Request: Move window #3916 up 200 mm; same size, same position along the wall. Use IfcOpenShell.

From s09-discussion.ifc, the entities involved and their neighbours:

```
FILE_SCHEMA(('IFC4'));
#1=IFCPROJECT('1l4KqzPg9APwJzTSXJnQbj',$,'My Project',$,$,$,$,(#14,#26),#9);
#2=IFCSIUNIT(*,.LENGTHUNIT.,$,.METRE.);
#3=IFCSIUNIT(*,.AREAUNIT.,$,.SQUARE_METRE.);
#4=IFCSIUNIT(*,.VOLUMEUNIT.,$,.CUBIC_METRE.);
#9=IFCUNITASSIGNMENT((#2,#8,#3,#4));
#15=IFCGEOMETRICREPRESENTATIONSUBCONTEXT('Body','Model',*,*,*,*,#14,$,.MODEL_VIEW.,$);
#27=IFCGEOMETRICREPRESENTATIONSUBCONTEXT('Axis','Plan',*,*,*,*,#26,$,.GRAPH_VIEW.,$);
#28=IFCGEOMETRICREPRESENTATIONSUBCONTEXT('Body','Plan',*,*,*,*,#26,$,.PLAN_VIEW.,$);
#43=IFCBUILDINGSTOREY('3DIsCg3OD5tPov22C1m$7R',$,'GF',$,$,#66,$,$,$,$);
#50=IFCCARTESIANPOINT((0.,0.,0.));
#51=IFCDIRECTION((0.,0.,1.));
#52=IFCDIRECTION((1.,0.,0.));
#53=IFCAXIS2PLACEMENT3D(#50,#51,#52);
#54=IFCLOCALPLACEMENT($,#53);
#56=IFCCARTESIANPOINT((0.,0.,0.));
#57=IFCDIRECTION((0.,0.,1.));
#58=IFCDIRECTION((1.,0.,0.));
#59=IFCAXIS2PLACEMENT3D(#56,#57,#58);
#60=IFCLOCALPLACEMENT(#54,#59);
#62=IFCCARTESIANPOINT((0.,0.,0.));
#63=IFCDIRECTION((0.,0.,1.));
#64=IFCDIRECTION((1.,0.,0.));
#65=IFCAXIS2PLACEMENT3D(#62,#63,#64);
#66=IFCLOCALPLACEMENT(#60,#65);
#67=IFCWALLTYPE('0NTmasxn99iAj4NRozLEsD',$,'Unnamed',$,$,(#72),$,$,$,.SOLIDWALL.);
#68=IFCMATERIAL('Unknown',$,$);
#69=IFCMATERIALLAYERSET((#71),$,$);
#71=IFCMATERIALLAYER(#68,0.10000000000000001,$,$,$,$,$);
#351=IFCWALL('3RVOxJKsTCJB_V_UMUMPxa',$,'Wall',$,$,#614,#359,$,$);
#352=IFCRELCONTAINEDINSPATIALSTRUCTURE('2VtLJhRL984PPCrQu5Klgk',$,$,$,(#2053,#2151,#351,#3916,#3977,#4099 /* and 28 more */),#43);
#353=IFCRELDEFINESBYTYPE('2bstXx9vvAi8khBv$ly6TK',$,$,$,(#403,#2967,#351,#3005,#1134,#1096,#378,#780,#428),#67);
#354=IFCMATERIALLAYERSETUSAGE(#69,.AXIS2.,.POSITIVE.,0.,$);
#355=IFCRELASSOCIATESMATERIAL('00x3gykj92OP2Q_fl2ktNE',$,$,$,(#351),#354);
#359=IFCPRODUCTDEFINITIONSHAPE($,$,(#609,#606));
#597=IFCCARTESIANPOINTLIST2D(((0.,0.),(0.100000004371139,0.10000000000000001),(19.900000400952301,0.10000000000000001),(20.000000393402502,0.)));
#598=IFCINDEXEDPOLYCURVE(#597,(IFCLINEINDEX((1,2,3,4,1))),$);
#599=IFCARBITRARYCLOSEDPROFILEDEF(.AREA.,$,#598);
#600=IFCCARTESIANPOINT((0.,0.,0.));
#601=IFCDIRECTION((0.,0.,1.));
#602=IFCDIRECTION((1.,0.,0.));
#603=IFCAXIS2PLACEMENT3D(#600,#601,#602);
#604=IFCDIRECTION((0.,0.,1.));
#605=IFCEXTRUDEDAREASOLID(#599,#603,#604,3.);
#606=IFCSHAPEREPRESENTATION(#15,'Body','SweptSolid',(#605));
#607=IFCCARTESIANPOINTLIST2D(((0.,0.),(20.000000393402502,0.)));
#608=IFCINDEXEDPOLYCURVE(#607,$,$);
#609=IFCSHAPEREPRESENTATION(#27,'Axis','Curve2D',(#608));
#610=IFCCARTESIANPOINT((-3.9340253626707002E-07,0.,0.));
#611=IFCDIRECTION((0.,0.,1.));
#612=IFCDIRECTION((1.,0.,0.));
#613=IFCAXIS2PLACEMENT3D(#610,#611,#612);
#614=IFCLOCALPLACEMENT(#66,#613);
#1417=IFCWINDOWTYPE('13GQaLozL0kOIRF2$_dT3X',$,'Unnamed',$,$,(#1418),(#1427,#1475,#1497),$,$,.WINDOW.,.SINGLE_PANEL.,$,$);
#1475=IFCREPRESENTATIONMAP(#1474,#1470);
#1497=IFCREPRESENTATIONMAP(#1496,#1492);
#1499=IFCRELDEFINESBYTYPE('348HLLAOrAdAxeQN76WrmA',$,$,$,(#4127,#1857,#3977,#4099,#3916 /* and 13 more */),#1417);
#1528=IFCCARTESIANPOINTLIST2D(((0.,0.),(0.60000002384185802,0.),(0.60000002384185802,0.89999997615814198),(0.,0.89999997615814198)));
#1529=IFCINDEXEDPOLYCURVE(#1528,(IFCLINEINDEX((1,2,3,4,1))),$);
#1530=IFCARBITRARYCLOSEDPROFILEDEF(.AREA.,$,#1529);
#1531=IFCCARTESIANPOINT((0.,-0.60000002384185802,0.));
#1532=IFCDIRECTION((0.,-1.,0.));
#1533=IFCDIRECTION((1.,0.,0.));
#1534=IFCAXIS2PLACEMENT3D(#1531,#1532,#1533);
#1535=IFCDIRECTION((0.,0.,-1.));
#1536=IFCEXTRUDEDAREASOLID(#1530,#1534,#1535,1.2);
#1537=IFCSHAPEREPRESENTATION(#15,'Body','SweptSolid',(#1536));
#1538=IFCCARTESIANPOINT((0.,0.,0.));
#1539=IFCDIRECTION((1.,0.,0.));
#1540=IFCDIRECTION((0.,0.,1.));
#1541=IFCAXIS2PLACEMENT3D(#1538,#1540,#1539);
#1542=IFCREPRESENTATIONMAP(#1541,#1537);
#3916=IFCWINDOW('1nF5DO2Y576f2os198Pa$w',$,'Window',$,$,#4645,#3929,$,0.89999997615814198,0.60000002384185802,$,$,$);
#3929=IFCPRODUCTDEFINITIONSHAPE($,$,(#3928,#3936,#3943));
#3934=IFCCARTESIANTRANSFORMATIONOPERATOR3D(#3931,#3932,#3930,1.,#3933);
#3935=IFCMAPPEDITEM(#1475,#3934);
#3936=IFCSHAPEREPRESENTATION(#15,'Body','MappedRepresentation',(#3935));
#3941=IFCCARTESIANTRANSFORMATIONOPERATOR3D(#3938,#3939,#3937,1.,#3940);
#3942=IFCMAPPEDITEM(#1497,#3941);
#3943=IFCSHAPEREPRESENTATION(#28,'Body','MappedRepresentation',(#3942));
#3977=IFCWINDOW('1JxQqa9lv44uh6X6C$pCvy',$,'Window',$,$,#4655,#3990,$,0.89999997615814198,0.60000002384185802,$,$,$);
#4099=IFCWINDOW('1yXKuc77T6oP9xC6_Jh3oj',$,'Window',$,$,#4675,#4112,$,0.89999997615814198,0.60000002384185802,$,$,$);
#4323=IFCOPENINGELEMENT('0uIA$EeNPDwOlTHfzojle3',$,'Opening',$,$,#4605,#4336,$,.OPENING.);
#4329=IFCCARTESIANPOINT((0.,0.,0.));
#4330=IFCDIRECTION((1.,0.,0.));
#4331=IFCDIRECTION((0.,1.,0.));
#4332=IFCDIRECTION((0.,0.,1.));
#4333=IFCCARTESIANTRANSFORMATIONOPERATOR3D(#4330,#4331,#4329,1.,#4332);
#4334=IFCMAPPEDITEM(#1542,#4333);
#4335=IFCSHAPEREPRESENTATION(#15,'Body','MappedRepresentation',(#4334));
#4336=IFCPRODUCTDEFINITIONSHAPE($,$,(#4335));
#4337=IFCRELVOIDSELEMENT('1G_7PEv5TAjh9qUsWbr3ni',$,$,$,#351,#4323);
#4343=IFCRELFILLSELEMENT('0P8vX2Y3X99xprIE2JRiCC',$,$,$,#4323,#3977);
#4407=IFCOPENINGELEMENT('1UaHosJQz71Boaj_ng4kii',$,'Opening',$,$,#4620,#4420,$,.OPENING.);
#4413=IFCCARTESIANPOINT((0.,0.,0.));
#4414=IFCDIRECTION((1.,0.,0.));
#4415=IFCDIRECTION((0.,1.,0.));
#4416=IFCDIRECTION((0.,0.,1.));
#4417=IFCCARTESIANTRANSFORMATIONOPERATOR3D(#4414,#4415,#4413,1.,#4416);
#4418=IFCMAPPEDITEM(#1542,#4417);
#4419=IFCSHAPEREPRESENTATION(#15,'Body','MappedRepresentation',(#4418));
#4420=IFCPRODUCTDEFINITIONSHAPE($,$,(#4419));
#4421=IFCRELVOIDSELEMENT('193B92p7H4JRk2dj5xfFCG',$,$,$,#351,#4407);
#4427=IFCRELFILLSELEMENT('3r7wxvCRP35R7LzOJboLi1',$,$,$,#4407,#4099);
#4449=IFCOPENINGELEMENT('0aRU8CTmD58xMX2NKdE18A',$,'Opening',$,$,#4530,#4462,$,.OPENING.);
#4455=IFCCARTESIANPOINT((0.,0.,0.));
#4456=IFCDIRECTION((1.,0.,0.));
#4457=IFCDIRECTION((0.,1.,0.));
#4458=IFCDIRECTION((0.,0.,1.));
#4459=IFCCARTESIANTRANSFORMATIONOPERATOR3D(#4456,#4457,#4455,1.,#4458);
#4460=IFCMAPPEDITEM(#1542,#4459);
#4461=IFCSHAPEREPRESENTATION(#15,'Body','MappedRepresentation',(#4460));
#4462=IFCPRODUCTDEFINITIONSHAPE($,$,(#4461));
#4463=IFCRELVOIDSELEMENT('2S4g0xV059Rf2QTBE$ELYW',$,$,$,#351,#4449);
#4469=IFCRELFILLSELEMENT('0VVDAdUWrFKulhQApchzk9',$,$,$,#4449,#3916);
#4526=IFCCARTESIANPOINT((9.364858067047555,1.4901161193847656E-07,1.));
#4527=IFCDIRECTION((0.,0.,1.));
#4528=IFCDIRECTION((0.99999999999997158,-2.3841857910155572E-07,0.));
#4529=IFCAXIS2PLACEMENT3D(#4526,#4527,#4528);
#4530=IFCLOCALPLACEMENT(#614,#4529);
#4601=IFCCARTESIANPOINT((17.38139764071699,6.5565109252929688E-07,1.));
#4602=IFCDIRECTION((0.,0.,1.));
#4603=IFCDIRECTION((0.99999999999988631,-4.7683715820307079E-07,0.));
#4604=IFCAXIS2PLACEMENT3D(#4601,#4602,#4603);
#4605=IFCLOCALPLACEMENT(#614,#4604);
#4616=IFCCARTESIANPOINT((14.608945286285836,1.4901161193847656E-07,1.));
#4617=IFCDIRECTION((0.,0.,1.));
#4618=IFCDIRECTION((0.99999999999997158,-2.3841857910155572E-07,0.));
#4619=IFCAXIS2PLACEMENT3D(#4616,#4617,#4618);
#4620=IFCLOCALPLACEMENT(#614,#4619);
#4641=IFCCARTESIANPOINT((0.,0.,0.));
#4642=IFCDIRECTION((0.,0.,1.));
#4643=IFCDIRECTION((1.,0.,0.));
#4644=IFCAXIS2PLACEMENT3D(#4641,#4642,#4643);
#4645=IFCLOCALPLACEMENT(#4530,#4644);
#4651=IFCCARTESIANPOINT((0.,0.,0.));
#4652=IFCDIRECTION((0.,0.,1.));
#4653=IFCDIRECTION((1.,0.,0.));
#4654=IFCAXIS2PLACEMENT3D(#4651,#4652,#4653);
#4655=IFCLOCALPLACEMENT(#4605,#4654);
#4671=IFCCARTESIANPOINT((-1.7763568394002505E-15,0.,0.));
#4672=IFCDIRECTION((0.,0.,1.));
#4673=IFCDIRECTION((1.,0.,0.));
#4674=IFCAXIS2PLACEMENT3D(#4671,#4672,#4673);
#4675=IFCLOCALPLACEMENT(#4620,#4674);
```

```python
import numpy as np
import ifcopenshell
import ifcopenshell.api.geometry
import ifcopenshell.util.placement
import ifcopenshell.util.unit

model = ifcopenshell.open("s09-discussion.ifc")
unit_scale = ifcopenshell.util.unit.calculate_unit_scale(model)

window = model.by_guid("1nF5DO2Y576f2os198Pa$w")
opening = window.FillsVoids[0].RelatingOpeningElement
dz = 0.2 / unit_scale

shift = np.array([0.0, 0.0, dz])
# The window is placed relative to its opening, so it follows when the opening moves.
matrix = ifcopenshell.util.placement.get_local_placement(opening.ObjectPlacement)
matrix[:3, 3] += shift
ifcopenshell.api.geometry.edit_object_placement(
    model, product=opening, matrix=matrix, is_si=False, should_transform_children=True
)

print(f"moved by {dz * unit_scale:+.3f} m")

model.write("s09-discussion_rev.ifc")
```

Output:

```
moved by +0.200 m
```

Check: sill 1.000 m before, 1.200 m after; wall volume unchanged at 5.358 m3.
